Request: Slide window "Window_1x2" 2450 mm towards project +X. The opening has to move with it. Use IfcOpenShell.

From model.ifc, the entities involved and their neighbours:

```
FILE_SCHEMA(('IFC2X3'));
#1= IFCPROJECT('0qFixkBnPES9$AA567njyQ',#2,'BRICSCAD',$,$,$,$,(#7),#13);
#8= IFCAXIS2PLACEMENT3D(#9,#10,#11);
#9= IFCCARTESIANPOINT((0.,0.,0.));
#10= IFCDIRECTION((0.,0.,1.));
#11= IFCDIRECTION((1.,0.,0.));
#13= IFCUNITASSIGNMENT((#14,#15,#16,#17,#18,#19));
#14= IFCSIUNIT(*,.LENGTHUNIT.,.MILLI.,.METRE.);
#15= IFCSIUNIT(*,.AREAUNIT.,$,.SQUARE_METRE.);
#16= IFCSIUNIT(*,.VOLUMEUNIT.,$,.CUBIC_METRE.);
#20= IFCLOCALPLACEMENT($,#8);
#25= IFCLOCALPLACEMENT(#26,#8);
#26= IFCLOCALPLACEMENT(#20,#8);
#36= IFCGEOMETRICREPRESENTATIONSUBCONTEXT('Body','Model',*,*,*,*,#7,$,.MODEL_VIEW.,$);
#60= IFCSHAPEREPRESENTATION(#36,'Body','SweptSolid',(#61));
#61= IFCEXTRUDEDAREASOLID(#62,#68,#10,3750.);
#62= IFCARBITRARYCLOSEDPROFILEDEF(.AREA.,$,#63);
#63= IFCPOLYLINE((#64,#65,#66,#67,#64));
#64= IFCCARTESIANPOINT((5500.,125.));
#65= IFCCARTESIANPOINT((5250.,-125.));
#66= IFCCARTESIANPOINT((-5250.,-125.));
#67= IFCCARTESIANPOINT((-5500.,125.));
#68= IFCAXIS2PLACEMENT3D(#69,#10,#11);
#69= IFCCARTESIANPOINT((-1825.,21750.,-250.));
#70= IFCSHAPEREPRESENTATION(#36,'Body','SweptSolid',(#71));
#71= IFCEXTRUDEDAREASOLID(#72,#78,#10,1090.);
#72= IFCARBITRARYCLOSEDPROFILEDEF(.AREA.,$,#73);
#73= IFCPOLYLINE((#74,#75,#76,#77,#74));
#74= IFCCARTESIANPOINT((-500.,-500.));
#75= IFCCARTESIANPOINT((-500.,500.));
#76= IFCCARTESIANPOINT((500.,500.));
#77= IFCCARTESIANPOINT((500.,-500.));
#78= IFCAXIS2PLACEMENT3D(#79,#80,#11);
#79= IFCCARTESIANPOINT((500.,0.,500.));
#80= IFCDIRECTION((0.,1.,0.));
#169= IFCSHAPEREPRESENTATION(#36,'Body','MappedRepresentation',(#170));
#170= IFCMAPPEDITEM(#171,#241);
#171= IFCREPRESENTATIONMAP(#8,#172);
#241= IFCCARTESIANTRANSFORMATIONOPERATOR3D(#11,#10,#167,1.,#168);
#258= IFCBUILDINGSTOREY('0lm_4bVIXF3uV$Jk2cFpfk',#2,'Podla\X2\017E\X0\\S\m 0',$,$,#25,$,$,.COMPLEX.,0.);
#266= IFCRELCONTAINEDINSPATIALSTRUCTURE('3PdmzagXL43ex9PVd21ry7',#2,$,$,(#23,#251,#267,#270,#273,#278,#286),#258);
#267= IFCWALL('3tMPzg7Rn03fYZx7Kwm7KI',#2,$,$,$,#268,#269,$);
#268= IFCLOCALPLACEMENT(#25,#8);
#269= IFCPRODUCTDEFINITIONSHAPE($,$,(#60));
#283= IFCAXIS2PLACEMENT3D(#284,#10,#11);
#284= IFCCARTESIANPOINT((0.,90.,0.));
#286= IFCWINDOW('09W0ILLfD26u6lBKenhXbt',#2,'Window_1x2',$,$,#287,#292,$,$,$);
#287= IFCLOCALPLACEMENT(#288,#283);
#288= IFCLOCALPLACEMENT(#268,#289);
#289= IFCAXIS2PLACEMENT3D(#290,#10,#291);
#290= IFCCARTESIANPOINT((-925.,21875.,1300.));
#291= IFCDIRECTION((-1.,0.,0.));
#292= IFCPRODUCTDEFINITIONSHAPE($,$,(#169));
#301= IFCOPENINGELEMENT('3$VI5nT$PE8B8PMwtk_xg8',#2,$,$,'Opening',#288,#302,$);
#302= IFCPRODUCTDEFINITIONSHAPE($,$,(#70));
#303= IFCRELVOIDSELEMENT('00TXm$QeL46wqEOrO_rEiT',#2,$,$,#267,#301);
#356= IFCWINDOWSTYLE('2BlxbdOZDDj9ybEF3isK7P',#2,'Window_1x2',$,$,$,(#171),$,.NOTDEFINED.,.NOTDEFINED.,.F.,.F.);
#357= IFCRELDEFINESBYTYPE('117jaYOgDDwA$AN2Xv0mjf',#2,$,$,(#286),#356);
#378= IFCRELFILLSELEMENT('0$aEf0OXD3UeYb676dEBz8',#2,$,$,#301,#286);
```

```python
import ifcopenshell
import ifcopenshell.api.geometry
import ifcopenshell.util.placement
import ifcopenshell.util.unit

model = ifcopenshell.open("model.ifc")
unit_scale = ifcopenshell.util.unit.calculate_unit_scale(model)

window = model.by_guid("09W0ILLfD26u6lBKenhXbt")
opening = window.FillsVoids[0].RelatingOpeningElement
wall = opening.VoidsElements[0].RelatingBuildingElement

wall_matrix = ifcopenshell.util.placement.get_local_placement(wall.ObjectPlacement)
shift = wall_matrix[:3, 0] * 2.45 / unit_scale
before = ifcopenshell.util.placement.get_local_placement(window.ObjectPlacement)[:3, 3].copy()

# The window is placed relative to its opening, so it follows when the opening moves.
matrix = ifcopenshell.util.placement.get_local_placement(opening.ObjectPlacement)
matrix[:3, 3] += shift
ifcopenshell.api.geometry.edit_object_placement(
    model, product=opening, matrix=matrix, is_si=False, should_transform_children=True
)

after = ifcopenshell.util.placement.get_local_placement(window.ObjectPlacement)[:3, 3]
print("window moved by", (after - before).round(3) + 0.0)

model.write("model_updated.ifc")
```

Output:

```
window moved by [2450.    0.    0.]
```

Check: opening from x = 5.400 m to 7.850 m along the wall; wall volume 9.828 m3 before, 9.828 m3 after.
